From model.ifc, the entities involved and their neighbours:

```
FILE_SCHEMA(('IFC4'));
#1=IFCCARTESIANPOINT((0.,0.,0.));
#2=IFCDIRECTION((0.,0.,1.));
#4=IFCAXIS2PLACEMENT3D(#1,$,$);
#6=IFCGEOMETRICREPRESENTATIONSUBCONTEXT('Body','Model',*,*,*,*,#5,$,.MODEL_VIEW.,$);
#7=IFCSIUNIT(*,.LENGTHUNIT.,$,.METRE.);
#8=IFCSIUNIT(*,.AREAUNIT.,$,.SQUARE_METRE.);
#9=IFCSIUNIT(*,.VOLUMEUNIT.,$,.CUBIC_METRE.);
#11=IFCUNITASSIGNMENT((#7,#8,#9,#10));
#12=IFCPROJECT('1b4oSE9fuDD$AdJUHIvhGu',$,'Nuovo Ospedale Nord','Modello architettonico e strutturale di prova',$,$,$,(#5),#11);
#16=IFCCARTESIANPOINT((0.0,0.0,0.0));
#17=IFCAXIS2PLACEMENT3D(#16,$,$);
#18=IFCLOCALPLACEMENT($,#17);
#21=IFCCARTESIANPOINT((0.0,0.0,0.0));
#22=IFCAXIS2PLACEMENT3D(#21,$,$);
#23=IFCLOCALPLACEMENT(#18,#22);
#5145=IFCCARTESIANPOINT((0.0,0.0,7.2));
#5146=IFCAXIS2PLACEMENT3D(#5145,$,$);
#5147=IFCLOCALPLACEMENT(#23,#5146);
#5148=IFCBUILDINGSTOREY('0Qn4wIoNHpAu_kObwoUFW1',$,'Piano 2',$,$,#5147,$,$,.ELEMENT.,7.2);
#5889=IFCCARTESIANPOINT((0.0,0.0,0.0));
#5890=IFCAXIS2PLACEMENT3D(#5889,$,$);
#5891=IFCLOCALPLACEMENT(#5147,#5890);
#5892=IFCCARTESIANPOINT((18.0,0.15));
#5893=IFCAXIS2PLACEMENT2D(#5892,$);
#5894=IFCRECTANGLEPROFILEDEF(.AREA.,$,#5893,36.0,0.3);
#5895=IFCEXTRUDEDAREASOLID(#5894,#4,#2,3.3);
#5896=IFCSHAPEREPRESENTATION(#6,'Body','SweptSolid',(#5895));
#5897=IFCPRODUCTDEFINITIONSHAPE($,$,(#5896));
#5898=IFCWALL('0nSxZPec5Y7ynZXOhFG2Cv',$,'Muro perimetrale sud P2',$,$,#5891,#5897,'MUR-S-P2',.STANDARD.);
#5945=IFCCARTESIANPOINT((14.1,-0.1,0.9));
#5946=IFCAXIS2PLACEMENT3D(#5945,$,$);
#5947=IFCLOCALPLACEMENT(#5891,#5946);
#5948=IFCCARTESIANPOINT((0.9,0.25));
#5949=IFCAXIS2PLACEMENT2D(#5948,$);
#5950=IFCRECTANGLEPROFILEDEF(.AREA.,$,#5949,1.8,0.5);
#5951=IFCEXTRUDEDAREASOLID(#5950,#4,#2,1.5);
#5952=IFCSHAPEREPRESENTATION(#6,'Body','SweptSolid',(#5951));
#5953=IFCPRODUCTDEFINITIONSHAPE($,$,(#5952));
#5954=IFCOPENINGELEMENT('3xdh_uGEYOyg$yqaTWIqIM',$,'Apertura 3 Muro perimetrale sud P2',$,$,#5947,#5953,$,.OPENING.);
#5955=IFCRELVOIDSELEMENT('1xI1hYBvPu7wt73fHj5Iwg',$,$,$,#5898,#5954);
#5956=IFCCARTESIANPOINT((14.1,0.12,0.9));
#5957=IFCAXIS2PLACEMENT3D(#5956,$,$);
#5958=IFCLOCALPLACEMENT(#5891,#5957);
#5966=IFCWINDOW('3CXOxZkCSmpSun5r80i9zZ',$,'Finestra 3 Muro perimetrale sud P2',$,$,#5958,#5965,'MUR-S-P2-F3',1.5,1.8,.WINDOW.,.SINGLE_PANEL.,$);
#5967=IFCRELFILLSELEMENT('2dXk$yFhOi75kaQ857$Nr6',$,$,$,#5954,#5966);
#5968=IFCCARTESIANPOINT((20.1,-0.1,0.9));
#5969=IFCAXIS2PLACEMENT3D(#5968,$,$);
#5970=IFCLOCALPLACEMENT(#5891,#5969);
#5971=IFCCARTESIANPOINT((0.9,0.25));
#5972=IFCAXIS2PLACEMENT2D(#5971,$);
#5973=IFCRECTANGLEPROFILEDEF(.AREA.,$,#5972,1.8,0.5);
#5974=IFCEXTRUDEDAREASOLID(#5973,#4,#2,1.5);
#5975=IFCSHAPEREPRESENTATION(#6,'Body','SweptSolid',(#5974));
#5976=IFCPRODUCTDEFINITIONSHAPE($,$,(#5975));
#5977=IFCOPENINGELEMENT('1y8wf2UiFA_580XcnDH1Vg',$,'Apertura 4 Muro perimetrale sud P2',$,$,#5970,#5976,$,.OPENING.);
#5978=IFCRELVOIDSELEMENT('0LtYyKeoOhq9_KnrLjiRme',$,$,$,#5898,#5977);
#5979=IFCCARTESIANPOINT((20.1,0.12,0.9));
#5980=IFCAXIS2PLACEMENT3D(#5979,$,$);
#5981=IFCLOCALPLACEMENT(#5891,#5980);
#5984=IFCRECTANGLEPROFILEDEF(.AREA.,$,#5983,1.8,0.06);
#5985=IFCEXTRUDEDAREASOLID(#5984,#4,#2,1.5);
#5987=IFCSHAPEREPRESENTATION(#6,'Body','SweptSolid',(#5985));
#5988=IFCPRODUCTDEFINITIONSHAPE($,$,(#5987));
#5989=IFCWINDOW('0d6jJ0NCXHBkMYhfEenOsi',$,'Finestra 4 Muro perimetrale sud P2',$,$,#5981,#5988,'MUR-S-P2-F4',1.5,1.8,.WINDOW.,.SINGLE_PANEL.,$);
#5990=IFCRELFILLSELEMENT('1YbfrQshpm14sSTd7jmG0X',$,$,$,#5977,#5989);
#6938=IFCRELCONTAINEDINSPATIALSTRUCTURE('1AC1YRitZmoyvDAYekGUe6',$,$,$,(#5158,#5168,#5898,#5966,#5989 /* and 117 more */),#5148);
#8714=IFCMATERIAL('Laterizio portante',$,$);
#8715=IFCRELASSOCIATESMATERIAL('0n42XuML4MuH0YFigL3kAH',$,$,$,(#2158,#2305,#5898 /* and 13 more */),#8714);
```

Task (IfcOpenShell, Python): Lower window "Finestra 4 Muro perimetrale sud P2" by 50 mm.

```python
import numpy as np
import ifcopenshell
import ifcopenshell.api.geometry
import ifcopenshell.util.placement
import ifcopenshell.util.unit

model = ifcopenshell.open("model.ifc")
unit_scale = ifcopenshell.util.unit.calculate_unit_scale(model)

window = model.by_guid("0d6jJ0NCXHBkMYhfEenOsi")
opening = window.FillsVoids[0].RelatingOpeningElement
dz = -0.05 / unit_scale

shift = np.array([0.0, 0.0, dz])
# The window is not placed relative to its opening, so move both.
for product in (opening, window):
    matrix = ifcopenshell.util.placement.get_local_placement(product.ObjectPlacement)
    matrix[:3, 3] += shift
    ifcopenshell.api.geometry.edit_object_placement(model, product=product, matrix=matrix, is_si=False)

print(f"moved by {dz * unit_scale:+.3f} m")

model.write("model_edited.ifc")
```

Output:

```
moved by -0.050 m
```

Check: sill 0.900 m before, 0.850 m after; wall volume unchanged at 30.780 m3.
